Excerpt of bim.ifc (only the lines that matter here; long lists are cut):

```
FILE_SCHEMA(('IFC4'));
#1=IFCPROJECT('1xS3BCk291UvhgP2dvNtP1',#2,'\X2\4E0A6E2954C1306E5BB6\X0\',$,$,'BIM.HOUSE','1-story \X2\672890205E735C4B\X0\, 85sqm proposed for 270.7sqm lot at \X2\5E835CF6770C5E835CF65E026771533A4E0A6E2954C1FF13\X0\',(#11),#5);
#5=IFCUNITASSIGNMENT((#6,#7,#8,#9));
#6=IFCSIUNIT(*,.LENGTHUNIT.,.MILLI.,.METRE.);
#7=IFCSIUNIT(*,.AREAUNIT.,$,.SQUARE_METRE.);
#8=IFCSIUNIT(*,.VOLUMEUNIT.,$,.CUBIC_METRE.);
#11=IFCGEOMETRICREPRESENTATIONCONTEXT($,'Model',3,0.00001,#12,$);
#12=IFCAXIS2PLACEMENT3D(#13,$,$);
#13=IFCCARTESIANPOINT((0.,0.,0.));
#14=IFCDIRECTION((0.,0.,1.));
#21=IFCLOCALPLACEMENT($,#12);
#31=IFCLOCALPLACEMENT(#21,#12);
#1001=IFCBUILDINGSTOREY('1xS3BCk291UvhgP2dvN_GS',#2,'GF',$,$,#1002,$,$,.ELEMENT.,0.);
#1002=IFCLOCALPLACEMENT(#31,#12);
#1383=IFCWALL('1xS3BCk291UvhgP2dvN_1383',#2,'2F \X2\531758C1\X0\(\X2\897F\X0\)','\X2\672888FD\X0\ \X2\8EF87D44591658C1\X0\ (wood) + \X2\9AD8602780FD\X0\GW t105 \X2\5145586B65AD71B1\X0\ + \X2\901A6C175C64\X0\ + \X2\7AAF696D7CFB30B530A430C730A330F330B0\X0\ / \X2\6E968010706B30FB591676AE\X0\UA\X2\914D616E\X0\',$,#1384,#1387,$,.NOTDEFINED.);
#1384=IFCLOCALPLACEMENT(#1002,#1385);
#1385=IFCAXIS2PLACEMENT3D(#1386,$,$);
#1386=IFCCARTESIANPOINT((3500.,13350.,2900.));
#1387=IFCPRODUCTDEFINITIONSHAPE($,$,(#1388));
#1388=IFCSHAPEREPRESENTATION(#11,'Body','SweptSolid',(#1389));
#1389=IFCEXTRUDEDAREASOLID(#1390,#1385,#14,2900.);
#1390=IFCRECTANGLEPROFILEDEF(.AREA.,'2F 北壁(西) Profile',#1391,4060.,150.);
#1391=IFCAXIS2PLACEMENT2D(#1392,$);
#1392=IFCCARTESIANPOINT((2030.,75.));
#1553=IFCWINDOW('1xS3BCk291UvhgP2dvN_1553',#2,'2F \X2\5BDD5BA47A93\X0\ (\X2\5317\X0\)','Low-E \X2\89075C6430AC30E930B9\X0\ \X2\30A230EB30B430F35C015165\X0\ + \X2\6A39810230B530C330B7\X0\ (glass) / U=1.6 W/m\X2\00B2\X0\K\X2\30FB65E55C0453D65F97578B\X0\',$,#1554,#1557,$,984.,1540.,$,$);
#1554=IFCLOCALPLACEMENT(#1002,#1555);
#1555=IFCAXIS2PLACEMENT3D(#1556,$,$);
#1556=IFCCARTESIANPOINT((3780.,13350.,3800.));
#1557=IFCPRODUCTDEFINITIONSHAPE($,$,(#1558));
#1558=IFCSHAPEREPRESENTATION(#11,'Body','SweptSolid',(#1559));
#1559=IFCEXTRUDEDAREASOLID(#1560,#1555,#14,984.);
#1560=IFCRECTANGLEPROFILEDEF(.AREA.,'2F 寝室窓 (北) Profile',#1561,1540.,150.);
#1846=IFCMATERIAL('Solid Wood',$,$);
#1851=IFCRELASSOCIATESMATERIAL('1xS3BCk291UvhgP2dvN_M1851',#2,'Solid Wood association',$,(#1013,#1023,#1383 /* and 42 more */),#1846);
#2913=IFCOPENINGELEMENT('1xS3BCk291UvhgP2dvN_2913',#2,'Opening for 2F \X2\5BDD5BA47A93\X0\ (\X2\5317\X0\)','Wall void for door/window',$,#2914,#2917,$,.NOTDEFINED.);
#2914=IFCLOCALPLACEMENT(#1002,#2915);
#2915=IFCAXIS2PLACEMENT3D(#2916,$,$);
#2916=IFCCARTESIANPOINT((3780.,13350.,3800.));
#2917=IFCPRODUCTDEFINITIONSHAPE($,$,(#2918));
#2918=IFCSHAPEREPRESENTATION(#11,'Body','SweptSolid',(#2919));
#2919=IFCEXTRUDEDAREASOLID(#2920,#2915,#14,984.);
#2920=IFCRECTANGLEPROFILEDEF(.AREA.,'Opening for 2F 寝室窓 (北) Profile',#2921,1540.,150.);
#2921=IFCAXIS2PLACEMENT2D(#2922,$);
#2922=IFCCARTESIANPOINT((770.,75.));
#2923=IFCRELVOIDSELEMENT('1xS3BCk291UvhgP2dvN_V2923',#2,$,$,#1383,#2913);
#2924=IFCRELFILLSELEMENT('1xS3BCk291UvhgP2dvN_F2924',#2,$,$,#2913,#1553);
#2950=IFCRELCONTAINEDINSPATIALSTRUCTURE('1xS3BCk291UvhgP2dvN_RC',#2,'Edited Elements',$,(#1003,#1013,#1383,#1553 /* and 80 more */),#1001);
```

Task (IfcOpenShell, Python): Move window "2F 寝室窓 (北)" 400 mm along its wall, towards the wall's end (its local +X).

```python
import ifcopenshell
import ifcopenshell.api.geometry
import ifcopenshell.util.placement

model = ifcopenshell.open("bim.ifc")

window = model.by_guid("1xS3BCk291UvhgP2dvN_1553")
opening = window.FillsVoids[0].RelatingOpeningElement
wall = opening.VoidsElements[0].RelatingBuildingElement

wall_matrix = ifcopenshell.util.placement.get_local_placement(wall.ObjectPlacement)
shift = wall_matrix[:3, 0] * 400.0
before = ifcopenshell.util.placement.get_local_placement(window.ObjectPlacement)[:3, 3].copy()

# The window is not placed relative to its opening, so move both.
for product in (opening, window):
    matrix = ifcopenshell.util.placement.get_local_placement(product.ObjectPlacement)
    matrix[:3, 3] += shift
    ifcopenshell.api.geometry.edit_object_placement(model, product=product, matrix=matrix, is_si=False)

after = ifcopenshell.util.placement.get_local_placement(window.ObjectPlacement)[:3, 3]
print("window moved by", (after - before).round(3) + 0.0)

model.write("bim_updated.ifc")
```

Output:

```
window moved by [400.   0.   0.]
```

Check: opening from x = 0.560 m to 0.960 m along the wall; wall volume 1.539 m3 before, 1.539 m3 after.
